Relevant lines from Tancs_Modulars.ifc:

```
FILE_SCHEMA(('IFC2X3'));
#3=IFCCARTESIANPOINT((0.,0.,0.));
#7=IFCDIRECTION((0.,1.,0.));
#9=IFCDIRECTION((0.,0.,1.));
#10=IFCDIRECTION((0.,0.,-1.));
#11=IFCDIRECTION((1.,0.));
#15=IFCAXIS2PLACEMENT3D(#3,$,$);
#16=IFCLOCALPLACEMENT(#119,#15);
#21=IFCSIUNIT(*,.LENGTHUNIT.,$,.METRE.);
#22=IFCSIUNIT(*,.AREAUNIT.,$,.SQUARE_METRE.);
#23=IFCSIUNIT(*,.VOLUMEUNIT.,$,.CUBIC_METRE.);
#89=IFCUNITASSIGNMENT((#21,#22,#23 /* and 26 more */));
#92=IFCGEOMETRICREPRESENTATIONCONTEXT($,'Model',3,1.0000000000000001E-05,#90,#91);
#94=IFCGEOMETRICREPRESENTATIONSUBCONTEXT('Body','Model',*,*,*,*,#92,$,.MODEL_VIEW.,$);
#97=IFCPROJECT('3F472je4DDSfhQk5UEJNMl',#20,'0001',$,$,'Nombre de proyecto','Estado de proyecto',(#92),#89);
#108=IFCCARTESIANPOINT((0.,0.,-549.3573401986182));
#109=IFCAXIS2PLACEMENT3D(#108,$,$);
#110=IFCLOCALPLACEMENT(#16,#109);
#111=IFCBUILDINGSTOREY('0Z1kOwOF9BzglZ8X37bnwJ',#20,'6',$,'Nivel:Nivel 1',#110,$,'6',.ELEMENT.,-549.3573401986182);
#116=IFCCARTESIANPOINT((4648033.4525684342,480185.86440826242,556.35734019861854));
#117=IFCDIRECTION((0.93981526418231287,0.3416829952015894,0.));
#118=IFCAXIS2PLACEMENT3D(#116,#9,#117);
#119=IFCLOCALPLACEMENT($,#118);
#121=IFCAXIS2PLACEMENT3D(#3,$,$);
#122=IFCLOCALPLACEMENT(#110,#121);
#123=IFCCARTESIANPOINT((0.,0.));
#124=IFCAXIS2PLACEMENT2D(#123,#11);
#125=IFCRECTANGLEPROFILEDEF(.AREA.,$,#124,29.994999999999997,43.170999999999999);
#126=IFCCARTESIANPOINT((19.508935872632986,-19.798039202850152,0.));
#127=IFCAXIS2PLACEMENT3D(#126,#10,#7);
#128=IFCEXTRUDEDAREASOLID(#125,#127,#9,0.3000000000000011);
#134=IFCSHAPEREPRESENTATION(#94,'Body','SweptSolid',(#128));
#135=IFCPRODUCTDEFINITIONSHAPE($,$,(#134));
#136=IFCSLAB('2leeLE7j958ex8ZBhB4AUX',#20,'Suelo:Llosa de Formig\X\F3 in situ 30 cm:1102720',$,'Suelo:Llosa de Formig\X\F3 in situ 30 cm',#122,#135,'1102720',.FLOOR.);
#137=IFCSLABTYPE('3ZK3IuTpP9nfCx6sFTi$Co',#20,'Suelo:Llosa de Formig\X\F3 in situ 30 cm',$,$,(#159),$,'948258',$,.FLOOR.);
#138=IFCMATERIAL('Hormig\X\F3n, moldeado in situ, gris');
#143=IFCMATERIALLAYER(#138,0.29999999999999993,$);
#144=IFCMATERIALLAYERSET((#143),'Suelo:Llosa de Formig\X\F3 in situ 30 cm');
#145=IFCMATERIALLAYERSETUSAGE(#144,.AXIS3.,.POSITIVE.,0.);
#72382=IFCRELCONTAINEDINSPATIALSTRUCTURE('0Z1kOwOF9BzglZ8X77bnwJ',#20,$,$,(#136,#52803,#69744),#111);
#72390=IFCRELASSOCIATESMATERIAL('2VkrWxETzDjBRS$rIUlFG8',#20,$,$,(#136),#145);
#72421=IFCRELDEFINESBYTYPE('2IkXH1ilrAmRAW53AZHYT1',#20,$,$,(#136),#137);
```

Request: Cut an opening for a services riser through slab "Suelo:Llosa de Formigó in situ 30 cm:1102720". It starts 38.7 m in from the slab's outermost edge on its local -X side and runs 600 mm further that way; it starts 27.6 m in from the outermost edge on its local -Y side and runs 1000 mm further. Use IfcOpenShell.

```python
import numpy as np
import ifcopenshell
import ifcopenshell.api.feature
import ifcopenshell.api.geometry
import ifcopenshell.api.root
import ifcopenshell.geom
import ifcopenshell.util.placement
import ifcopenshell.util.representation
import ifcopenshell.util.shape
import ifcopenshell.util.unit

model = ifcopenshell.open("Tancs_Modulars.ifc")
unit_scale = ifcopenshell.util.unit.calculate_unit_scale(model)
settings = ifcopenshell.geom.settings()


def volume(element):
    """Net volume in cubic metres, openings subtracted."""
    shape = ifcopenshell.geom.create_shape(settings, element)
    return ifcopenshell.util.shape.get_volume(shape.geometry)


slab = model.by_guid("2leeLE7j958ex8ZBhB4AUX")
before = volume(slab)

# Extent in the slab's own axes, in metres. The edges named are its -X and -Y sides.
slab_shape = ifcopenshell.geom.create_shape(settings, slab)
vertices = ifcopenshell.util.shape.get_vertices(slab_shape.geometry)
x_min, y_min, bottom = vertices.min(axis=0)
top = vertices[:, 2].max()

opening = ifcopenshell.api.root.create_entity(model, ifc_class="IfcOpeningElement", name="Services riser opening")
context = ifcopenshell.util.representation.get_context(model, "Model", "Body", "MODEL_VIEW")
width, depth = 0.6, 1
outline = [(0.0, 0.0), (width, 0.0), (width, depth), (0.0, depth), (0.0, 0.0)]
# Overshoot both faces by 50 mm so the cut is clean.
shape = ifcopenshell.api.geometry.add_slab_representation(
    model, context=context, depth=top - bottom + 0.1, polyline=outline
)
ifcopenshell.api.geometry.assign_representation(model, product=opening, representation=shape)

matrix = ifcopenshell.util.placement.get_local_placement(slab.ObjectPlacement)
matrix[:, 3] = matrix @ np.append(np.array([x_min + 38.7, y_min + 27.6, bottom - 0.05]) / unit_scale, 1.0)
ifcopenshell.api.geometry.edit_object_placement(model, product=opening, matrix=matrix, is_si=False)
ifcopenshell.api.feature.add_feature(model, feature=opening, element=slab)

after = volume(slab)

print(f"slab volume {before:.3f} -> {after:.3f} m3")

model.write("Tancs_Modulars_rev.ifc")
```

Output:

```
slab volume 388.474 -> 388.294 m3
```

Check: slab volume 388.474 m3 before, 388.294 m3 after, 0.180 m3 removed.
